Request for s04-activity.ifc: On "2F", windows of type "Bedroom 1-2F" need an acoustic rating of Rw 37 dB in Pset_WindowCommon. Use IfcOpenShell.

First a look at what the model holds.

```python
import ifcopenshell
import ifcopenshell.util.element

model = ifcopenshell.open("s04-activity.ifc")
print(model.schema)
storey = next(s for s in model.by_type("IfcBuildingStorey") if s.Name == "2F")
windows = [e for e in ifcopenshell.util.element.get_decomposition(storey) if e.is_a("IfcWindow")]
seen = {}
for e in windows:
    element_type = ifcopenshell.util.element.get_type(e)
    key = (element_type.Name if element_type != e and element_type else None, ifcopenshell.util.element.get_pset(e, "Pset_WindowCommon", "AcousticRating"))
    seen[key] = seen.get(key, 0) + 1
for (name, value), count in sorted(seen.items(), key=str):
    print(count, "x", name, "|", value)
```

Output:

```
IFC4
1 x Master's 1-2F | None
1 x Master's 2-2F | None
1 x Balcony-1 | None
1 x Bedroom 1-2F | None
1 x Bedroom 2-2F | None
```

```python
import ifcopenshell
import ifcopenshell.api.pset
import ifcopenshell.util.element

model = ifcopenshell.open("s04-activity.ifc")

storey = next(s for s in model.by_type("IfcBuildingStorey") if s.Name == "2F")
windows = [e for e in ifcopenshell.util.element.get_decomposition(storey) if e.is_a("IfcWindow")]

count = 0
for e in windows:
    element_type = ifcopenshell.util.element.get_type(e)
    if element_type in (None, e) or element_type.Name != "Bedroom 1-2F":
        continue
    # add_pset returns the element's existing set when there is one.
    pset = ifcopenshell.api.pset.add_pset(model, product=e, name="Pset_WindowCommon")
    ifcopenshell.api.pset.edit_pset(model, pset=pset, properties={"AcousticRating": "Rw 37 dB"})
    count += 1

print(count, "windows updated")

model.write("s04-activity_v2.ifc")
```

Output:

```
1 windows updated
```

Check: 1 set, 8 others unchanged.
